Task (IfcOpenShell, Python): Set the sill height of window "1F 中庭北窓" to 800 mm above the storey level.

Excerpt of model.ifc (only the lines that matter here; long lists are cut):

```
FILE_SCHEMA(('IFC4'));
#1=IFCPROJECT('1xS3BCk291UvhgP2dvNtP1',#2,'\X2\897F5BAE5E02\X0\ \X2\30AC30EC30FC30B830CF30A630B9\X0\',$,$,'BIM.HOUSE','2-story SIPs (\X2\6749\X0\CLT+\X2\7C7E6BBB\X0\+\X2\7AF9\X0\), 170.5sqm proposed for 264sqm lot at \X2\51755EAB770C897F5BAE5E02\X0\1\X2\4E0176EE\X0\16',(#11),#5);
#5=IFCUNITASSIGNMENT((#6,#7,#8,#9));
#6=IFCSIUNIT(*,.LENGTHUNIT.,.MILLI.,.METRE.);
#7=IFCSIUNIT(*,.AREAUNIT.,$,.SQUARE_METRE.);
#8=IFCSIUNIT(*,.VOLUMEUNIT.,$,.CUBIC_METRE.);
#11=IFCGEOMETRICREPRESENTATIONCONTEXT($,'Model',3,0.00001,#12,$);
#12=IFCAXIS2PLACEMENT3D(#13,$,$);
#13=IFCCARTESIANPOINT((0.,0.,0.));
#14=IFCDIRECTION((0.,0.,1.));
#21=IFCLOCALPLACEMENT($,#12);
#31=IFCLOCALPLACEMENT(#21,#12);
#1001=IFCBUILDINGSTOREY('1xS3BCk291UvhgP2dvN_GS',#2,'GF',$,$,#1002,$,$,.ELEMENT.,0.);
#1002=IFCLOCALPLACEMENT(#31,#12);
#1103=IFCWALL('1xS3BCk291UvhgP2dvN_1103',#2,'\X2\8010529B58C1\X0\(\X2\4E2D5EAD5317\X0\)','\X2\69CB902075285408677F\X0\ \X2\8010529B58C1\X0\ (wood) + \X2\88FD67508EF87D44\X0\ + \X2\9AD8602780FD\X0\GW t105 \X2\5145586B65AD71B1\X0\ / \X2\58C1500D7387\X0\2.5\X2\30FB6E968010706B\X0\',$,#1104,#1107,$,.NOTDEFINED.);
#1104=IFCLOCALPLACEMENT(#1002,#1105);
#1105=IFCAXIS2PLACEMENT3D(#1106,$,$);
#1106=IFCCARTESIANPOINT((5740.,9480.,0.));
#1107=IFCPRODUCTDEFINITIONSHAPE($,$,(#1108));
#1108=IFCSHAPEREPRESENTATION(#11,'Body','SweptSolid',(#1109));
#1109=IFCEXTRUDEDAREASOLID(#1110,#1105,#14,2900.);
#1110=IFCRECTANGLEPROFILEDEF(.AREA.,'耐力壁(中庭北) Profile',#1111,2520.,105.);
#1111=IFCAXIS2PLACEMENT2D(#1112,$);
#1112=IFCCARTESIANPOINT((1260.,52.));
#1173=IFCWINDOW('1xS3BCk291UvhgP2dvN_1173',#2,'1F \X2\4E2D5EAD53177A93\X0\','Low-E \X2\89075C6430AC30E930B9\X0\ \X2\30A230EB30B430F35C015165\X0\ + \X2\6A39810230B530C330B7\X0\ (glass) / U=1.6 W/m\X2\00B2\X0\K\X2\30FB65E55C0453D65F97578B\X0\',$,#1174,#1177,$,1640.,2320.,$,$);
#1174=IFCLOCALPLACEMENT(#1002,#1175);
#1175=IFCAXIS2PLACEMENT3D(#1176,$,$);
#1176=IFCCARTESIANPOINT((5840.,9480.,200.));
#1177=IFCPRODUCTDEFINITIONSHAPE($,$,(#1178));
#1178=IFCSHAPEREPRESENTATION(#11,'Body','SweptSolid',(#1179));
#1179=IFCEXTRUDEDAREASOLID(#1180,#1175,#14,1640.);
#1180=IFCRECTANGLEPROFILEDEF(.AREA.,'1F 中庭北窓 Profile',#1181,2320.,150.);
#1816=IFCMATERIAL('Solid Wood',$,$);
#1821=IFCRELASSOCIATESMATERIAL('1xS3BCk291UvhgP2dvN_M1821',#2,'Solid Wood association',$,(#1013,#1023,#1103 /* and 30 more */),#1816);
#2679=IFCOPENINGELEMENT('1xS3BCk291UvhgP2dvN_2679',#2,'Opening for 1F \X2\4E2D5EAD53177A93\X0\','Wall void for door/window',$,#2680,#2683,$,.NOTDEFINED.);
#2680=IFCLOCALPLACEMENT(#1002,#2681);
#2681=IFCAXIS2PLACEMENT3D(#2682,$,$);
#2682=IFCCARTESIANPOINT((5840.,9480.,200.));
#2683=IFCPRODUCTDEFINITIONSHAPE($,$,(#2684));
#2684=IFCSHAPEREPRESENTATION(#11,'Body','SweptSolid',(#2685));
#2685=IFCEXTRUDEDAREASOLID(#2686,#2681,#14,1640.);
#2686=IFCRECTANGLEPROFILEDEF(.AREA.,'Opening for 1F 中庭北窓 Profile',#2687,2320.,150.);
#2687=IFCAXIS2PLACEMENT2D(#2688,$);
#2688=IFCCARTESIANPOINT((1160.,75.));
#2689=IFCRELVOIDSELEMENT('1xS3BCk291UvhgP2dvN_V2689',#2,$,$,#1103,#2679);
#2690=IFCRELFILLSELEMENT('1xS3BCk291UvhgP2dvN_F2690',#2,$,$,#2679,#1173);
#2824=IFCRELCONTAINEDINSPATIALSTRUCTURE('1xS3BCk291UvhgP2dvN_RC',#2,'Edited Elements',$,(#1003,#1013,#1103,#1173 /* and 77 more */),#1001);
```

```python
import numpy as np
import ifcopenshell
import ifcopenshell.api.geometry
import ifcopenshell.geom
import ifcopenshell.util.element
import ifcopenshell.util.placement
import ifcopenshell.util.shape
import ifcopenshell.util.unit

model = ifcopenshell.open("model.ifc")
unit_scale = ifcopenshell.util.unit.calculate_unit_scale(model)

window = model.by_id(1173)
opening = window.FillsVoids[0].RelatingOpeningElement
storey = ifcopenshell.util.element.get_container(window, ifc_class="IfcBuildingStorey")
level = ifcopenshell.util.placement.get_local_placement(storey.ObjectPlacement)[2, 3]

# The opening's origin need not be at the sill, so measure its lowest point.
shape = ifcopenshell.geom.create_shape(ifcopenshell.geom.settings(), opening)
bottom = ifcopenshell.util.shape.get_shape_bottom_elevation(shape, shape.geometry) / unit_scale
dz = level + 800.0 - bottom

shift = np.array([0.0, 0.0, dz])
# The window is not placed relative to its opening, so move both.
for product in (opening, window):
    matrix = ifcopenshell.util.placement.get_local_placement(product.ObjectPlacement)
    matrix[:3, 3] += shift
    ifcopenshell.api.geometry.edit_object_placement(model, product=product, matrix=matrix, is_si=False)

print(f"moved by {dz * unit_scale:+.3f} m")

model.write("model-out.ifc")
```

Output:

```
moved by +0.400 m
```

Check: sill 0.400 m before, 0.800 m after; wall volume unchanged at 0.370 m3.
